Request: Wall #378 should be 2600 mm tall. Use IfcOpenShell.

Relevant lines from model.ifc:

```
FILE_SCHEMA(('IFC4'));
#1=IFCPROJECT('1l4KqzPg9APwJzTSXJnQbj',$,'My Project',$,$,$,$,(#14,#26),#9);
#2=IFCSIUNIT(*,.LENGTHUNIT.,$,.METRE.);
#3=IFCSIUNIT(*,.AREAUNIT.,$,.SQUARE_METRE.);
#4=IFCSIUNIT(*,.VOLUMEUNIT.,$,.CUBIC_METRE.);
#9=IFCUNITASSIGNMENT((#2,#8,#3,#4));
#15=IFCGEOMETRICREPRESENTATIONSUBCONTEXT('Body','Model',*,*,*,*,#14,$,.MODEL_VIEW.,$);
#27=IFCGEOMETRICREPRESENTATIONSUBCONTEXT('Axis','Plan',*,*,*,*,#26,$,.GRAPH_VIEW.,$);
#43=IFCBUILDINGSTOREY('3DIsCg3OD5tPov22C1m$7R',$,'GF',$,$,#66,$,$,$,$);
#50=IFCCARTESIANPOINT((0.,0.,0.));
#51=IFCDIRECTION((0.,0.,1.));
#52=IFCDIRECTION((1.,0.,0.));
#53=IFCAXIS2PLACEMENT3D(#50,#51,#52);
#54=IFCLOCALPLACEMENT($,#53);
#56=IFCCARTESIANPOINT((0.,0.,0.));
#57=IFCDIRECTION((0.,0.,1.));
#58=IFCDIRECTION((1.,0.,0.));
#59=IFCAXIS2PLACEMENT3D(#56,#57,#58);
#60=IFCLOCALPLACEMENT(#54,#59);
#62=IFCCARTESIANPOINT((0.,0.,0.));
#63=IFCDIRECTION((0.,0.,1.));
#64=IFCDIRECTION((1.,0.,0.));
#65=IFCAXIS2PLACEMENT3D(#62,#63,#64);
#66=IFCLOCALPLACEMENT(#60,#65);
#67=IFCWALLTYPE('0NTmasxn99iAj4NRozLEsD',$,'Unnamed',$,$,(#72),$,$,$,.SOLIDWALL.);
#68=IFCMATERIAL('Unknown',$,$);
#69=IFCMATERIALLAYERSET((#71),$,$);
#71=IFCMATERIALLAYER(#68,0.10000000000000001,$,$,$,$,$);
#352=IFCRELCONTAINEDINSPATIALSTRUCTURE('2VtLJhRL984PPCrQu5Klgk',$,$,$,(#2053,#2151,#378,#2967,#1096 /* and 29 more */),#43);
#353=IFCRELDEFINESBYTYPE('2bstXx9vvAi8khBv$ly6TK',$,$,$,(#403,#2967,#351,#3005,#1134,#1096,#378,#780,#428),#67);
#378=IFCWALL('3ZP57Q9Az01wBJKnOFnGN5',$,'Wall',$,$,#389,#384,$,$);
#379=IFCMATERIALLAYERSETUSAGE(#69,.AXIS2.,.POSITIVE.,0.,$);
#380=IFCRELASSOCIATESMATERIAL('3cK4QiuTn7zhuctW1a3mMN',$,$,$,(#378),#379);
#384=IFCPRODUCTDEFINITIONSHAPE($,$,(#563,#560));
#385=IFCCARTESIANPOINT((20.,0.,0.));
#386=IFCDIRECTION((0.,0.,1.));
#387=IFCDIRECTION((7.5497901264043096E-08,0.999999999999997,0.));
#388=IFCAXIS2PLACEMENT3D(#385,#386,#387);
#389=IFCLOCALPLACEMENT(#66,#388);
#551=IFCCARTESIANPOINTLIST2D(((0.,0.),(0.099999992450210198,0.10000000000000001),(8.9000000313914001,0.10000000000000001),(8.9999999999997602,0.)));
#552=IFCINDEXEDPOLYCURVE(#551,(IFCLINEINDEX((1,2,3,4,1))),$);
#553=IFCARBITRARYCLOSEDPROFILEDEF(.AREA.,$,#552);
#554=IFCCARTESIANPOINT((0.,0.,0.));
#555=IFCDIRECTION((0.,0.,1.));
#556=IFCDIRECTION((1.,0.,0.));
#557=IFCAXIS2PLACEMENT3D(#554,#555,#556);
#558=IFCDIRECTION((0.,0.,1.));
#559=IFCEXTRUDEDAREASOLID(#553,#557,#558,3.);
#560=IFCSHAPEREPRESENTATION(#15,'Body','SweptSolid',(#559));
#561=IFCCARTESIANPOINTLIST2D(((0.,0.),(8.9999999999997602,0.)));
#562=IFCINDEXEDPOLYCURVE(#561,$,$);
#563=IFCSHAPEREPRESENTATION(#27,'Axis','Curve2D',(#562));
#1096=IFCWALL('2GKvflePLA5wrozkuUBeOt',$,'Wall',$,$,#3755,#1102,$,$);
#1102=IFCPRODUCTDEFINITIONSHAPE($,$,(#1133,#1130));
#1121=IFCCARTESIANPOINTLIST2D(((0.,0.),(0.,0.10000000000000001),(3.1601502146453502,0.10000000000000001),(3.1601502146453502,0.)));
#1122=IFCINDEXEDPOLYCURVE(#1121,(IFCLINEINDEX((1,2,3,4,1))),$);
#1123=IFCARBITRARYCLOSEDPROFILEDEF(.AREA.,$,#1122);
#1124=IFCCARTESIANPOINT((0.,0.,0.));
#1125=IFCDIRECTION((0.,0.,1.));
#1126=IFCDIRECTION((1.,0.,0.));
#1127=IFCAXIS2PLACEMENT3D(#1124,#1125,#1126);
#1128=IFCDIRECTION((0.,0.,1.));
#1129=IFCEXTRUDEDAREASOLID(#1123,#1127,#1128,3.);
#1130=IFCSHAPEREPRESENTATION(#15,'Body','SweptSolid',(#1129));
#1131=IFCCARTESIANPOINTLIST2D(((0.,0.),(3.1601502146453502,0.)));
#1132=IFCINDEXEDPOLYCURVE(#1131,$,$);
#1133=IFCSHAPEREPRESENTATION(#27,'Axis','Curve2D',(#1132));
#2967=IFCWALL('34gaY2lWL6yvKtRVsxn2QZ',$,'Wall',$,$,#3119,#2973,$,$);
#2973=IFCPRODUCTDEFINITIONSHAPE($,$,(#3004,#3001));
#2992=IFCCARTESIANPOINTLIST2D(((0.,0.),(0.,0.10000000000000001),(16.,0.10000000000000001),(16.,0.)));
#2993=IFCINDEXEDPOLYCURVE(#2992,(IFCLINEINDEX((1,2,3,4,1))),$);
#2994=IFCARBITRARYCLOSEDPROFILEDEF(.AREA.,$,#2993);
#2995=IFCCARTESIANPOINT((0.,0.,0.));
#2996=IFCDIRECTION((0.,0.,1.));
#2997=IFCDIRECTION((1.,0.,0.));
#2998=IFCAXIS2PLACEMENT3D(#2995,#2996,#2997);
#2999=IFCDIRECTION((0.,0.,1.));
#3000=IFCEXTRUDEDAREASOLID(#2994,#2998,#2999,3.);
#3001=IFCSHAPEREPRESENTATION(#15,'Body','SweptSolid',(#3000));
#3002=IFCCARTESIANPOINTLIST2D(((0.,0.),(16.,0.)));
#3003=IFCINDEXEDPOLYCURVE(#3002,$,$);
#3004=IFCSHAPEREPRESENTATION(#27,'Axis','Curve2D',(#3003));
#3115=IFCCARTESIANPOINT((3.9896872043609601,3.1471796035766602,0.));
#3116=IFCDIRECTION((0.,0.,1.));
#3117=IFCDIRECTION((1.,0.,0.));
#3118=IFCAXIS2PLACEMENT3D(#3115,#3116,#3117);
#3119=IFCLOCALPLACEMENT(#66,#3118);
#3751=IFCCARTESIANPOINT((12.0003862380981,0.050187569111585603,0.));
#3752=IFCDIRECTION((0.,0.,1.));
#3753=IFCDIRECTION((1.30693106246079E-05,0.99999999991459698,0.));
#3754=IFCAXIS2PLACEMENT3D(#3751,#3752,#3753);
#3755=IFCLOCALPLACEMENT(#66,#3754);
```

```python
import ifcopenshell
import ifcopenshell.geom
import ifcopenshell.util.representation
import ifcopenshell.util.shape
import ifcopenshell.util.unit

model = ifcopenshell.open("model.ifc")
unit_scale = ifcopenshell.util.unit.calculate_unit_scale(model)
settings = ifcopenshell.geom.settings()


def volume(element):
    """Net volume in cubic metres, openings subtracted."""
    shape = ifcopenshell.geom.create_shape(settings, element)
    return ifcopenshell.util.shape.get_volume(shape.geometry)


wall = model.by_id(378)
before = volume(wall)

body = ifcopenshell.util.representation.get_representation(wall, "Model", "Body")
solid = body.Items[0]
old_height = solid.Depth
solid.Depth = 2.6 / unit_scale
after = volume(wall)

print(f"height {old_height:g} -> {solid.Depth:g}, volume {before:.3f} -> {after:.3f} m3")

model.write("model_updated.ifc")
```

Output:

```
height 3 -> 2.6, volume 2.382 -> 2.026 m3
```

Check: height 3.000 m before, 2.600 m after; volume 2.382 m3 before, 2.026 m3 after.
